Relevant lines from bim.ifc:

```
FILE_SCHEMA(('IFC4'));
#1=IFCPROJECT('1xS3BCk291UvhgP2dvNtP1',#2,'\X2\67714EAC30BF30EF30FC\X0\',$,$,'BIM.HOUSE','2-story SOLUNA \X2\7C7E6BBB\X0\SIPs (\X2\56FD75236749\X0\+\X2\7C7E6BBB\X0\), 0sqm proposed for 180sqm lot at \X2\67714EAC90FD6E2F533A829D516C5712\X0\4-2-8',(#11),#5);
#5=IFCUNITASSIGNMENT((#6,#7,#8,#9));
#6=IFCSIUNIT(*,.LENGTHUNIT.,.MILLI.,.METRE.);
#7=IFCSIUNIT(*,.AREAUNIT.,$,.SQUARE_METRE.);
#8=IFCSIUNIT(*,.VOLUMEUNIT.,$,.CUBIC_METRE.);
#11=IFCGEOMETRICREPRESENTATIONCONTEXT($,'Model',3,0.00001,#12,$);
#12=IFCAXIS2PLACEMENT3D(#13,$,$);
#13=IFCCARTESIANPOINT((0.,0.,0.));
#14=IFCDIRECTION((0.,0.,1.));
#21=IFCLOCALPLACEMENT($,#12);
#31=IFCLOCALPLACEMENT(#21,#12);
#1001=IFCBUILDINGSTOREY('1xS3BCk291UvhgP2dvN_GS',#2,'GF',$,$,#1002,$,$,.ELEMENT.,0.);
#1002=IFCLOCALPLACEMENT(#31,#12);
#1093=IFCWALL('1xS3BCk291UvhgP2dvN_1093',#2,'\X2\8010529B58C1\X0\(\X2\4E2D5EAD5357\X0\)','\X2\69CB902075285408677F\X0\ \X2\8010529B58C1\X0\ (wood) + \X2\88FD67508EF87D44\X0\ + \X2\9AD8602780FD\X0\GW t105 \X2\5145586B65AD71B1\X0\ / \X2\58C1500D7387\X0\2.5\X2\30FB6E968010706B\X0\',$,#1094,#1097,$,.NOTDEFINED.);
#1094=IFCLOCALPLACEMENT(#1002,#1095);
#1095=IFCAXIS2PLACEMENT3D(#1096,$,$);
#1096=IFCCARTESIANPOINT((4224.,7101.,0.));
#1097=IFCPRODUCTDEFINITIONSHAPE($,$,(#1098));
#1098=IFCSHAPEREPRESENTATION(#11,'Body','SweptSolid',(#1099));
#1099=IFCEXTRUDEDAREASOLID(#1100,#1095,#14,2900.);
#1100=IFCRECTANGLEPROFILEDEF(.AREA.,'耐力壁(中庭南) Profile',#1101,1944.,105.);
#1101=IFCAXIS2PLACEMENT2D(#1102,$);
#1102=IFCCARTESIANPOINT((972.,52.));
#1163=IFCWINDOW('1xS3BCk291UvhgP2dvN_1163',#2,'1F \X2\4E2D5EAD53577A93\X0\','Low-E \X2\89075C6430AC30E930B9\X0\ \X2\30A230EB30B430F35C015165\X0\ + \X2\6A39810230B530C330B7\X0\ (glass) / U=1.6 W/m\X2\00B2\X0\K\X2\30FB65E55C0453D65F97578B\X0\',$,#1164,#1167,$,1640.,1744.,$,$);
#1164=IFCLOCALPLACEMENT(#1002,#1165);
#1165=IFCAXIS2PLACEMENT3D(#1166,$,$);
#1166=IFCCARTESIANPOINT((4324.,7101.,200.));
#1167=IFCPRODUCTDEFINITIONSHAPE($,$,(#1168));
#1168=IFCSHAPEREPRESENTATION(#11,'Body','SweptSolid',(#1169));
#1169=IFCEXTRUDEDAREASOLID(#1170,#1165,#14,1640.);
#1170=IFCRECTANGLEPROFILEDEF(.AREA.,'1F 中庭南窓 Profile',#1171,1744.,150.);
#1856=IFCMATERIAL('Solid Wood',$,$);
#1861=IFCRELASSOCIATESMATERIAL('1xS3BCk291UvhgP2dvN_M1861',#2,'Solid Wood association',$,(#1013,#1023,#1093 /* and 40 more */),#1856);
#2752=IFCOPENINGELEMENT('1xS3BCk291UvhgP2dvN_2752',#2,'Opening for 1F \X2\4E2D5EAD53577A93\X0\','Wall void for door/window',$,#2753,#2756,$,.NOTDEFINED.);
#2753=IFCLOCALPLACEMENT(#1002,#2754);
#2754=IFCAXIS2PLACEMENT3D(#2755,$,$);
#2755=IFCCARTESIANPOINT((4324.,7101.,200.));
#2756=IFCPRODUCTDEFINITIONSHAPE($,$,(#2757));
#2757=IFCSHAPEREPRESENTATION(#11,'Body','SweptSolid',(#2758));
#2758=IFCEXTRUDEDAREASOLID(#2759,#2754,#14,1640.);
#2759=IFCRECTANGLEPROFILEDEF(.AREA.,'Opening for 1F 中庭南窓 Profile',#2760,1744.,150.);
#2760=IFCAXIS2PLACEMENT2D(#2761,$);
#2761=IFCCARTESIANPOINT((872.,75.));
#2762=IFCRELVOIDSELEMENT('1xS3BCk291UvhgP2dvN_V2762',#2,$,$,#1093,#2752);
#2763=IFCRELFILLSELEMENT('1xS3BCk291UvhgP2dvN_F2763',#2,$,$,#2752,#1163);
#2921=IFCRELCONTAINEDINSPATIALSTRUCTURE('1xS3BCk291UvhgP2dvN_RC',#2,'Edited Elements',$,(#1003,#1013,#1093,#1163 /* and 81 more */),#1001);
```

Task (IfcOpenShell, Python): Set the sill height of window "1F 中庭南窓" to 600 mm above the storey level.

```python
import numpy as np
import ifcopenshell
import ifcopenshell.api.geometry
import ifcopenshell.geom
import ifcopenshell.util.element
import ifcopenshell.util.placement
import ifcopenshell.util.shape
import ifcopenshell.util.unit

model = ifcopenshell.open("bim.ifc")
unit_scale = ifcopenshell.util.unit.calculate_unit_scale(model)

window = model.by_id(1163)
opening = window.FillsVoids[0].RelatingOpeningElement
storey = ifcopenshell.util.element.get_container(window, ifc_class="IfcBuildingStorey")
level = ifcopenshell.util.placement.get_local_placement(storey.ObjectPlacement)[2, 3]

# The opening's origin need not be at the sill, so measure its lowest point.
shape = ifcopenshell.geom.create_shape(ifcopenshell.geom.settings(), opening)
bottom = ifcopenshell.util.shape.get_shape_bottom_elevation(shape, shape.geometry) / unit_scale
dz = level + 0.6 / unit_scale - bottom

shift = np.array([0.0, 0.0, dz])
# The window is not placed relative to its opening, so move both.
for product in (opening, window):
    matrix = ifcopenshell.util.placement.get_local_placement(product.ObjectPlacement)
    matrix[:3, 3] += shift
    ifcopenshell.api.geometry.edit_object_placement(model, product=product, matrix=matrix, is_si=False)

print(f"moved by {dz * unit_scale:+.3f} m")

model.write("bim_edited.ifc")
```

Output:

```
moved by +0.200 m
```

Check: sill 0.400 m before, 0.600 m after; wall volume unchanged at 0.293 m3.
